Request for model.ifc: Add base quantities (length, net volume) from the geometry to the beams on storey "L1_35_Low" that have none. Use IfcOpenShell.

First a look at what the model holds.

```python
import ifcopenshell
import ifcopenshell.util.element
import ifcopenshell.util.unit

model = ifcopenshell.open("model.ifc")
print(model.schema)
for unit_type in ("LENGTHUNIT", "AREAUNIT", "VOLUMEUNIT"):
    print(unit_type, ifcopenshell.util.unit.calculate_unit_scale(model, unit_type))
storey = next(s for s in model.by_type("IfcBuildingStorey") if s.Name == "L1_35_Low")
beams = [e for e in ifcopenshell.util.element.get_decomposition(storey) if e.is_a("IfcBeam")]
for e in sorted(beams, key=lambda e: e.id()):
    print(e.id(), e.is_a(), e.Name, list(ifcopenshell.util.element.get_psets(e, qtos_only=True)), sep=" | ")
```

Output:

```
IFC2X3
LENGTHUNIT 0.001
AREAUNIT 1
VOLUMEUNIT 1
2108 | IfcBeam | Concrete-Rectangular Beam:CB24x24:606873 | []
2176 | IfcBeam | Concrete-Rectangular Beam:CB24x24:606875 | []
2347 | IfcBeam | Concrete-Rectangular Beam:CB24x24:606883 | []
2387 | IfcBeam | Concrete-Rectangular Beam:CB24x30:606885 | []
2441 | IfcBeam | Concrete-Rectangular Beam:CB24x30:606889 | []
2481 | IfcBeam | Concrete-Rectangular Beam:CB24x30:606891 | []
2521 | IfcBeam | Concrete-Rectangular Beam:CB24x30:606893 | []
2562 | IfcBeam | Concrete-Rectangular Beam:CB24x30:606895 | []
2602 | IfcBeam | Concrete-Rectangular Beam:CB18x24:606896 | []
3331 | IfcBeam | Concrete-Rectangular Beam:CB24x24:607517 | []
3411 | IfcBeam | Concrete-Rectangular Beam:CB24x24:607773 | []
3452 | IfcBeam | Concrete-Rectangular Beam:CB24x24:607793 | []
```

```python
import ifcopenshell
import ifcopenshell.api.pset
import ifcopenshell.geom
import ifcopenshell.util.element
import ifcopenshell.util.shape
import ifcopenshell.util.unit

model = ifcopenshell.open("model.ifc")
unit_scale = ifcopenshell.util.unit.calculate_unit_scale(model)
volume_scale = ifcopenshell.util.unit.calculate_unit_scale(model, "VOLUMEUNIT")
settings = ifcopenshell.geom.settings()

storey = next(s for s in model.by_type("IfcBuildingStorey") if s.Name == "L1_35_Low")
beams = [e for e in ifcopenshell.util.element.get_decomposition(storey) if e.is_a("IfcBeam")]

for e in sorted(beams, key=lambda e: e.id()):
    if ifcopenshell.util.element.get_psets(e, qtos_only=True, should_inherit=False):
        continue
    # Geometry comes back in metres, in the element's own axes.
    shape = ifcopenshell.geom.create_shape(settings, e)
    values = {
        "Length": ifcopenshell.util.shape.get_max_xyz(shape.geometry) / unit_scale,
        "NetVolume": ifcopenshell.util.shape.get_volume(shape.geometry) / volume_scale,
    }
    qto = ifcopenshell.api.pset.add_qto(model, product=e, name="BaseQuantities")
    ifcopenshell.api.pset.edit_qto(model, qto=qto, properties=values)
    print(e.id(), {k: round(v, 3) for k, v in values.items()})

model.write("model_rev.ifc")
```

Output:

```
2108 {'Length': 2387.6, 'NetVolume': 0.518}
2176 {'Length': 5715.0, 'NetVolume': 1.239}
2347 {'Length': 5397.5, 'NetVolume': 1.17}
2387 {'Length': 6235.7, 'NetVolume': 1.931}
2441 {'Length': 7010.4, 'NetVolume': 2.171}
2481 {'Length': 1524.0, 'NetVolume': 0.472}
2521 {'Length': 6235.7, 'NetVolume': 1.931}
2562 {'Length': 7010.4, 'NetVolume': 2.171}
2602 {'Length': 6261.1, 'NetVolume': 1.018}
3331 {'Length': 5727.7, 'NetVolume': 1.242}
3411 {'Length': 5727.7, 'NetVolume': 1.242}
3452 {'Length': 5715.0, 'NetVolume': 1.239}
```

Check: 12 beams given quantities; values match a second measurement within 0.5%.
